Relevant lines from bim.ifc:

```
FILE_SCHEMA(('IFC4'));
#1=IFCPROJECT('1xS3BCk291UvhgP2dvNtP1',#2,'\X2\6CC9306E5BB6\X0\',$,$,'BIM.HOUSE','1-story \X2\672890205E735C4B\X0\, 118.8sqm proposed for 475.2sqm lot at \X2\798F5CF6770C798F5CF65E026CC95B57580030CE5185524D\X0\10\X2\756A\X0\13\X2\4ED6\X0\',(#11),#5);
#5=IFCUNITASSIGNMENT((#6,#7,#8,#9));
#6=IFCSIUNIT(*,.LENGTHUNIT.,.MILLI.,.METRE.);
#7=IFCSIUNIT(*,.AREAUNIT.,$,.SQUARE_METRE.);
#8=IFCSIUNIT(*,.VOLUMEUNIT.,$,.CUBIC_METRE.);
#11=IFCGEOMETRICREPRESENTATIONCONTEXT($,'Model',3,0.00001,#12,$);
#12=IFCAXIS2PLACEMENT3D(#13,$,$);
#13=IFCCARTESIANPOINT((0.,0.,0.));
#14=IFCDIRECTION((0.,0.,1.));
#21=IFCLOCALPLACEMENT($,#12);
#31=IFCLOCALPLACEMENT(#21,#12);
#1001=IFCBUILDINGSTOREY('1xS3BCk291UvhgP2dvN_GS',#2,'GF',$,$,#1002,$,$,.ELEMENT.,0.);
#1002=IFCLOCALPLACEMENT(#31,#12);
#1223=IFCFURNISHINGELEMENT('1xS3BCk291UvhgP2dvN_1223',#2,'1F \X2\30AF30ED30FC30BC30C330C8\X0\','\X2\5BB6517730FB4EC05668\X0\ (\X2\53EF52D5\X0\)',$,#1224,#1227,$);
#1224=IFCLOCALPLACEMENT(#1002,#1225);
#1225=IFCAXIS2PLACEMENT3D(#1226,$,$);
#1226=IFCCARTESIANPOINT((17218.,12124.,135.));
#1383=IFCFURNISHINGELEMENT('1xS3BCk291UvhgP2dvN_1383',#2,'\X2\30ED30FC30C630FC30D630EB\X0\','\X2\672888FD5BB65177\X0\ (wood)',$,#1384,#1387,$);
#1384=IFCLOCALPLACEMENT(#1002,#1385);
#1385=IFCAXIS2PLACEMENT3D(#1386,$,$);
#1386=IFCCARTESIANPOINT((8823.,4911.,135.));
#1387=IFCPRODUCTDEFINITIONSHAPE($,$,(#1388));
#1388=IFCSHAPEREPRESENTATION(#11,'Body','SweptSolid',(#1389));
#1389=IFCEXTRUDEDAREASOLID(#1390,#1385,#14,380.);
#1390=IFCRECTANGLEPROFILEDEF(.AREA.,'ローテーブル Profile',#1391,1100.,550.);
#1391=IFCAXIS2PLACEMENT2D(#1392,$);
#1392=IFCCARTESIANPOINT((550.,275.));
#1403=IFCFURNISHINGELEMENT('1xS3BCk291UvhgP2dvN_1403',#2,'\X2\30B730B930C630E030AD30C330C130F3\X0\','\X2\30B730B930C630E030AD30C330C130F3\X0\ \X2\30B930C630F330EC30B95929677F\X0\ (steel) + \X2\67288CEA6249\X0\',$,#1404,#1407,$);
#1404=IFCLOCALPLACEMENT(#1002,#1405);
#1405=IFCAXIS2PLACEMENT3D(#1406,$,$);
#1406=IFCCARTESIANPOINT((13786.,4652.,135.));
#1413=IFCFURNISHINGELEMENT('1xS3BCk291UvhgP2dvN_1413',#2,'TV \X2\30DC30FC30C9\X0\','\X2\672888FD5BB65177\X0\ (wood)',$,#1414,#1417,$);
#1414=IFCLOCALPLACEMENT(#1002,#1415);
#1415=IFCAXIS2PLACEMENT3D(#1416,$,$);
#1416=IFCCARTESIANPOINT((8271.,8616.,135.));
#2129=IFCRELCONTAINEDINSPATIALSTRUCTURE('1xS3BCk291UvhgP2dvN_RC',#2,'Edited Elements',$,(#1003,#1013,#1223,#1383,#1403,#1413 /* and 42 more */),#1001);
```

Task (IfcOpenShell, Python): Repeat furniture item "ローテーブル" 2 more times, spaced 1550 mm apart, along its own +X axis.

```python
import ifcopenshell
import ifcopenshell.api.geometry
import ifcopenshell.api.root
import ifcopenshell.util.element
import ifcopenshell.util.placement

model = ifcopenshell.open("bim.ifc")


def reuse_history(source, copy):
    """copy_class also copies each property set's owner history, people and application; keep the originals."""
    for rel in copy.IsDefinedBy:
        if rel.is_a("IfcRelDefinesByProperties") and (history := rel.RelatingPropertyDefinition.OwnerHistory):
            rel.RelatingPropertyDefinition.OwnerHistory = source.OwnerHistory
            ifcopenshell.util.element.remove_deep2(model, history)


source = model.by_guid("1xS3BCk291UvhgP2dvN_1383")
base = ifcopenshell.util.placement.get_local_placement(source.ObjectPlacement)
step = base[:3, 0] * 1550.0

for i in range(1, 3):
    copy = ifcopenshell.api.root.copy_class(model, product=source)
    copy.Representation = ifcopenshell.util.element.copy_deep(
        model, source.Representation, exclude=["IfcGeometricRepresentationContext", "IfcRepresentationMap"]
    )
    reuse_history(source, copy)
    matrix = base.copy()
    matrix[:3, 3] += i * step
    print("added at", matrix[:3, 3].round(3) + 0.0)
    ifcopenshell.api.geometry.edit_object_placement(model, product=copy, matrix=matrix, is_si=False)

model.write("bim_edited.ifc")
```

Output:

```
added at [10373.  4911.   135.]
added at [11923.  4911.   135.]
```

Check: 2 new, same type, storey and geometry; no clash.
